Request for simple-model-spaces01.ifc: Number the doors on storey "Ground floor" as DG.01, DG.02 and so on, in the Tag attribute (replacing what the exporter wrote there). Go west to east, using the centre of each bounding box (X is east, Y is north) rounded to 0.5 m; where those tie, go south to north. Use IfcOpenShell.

First a look at what the model holds.

```python
import ifcopenshell
import ifcopenshell.util.element
import ifcopenshell.util.placement

model = ifcopenshell.open("simple-model-spaces01.ifc")
print(model.schema)
storey = next(s for s in model.by_type("IfcBuildingStorey") if s.Name == "Ground floor")
doors = [e for e in ifcopenshell.util.element.get_decomposition(storey) if e.is_a("IfcDoor")]
for e in sorted(doors, key=lambda e: e.id()):
    origin = ifcopenshell.util.placement.get_local_placement(e.ObjectPlacement)[:3, 3]
    print(e.id(), e.Tag, e.Name, origin.round(2) + 0.0, sep=" | ")
```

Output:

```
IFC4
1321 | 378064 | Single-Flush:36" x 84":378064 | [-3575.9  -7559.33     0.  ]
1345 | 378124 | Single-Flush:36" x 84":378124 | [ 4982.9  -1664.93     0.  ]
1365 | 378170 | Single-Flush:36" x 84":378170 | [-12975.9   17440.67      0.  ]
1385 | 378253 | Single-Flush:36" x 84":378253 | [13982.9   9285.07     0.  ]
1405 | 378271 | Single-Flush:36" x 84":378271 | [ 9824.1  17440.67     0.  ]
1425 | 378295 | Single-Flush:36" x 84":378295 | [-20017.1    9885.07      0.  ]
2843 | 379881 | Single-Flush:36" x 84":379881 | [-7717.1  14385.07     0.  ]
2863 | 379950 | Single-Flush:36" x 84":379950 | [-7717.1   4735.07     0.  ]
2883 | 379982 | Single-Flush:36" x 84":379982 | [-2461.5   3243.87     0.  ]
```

```python
import ifcopenshell
import ifcopenshell.geom
import ifcopenshell.util.element
import ifcopenshell.util.shape

model = ifcopenshell.open("simple-model-spaces01.ifc")
settings = ifcopenshell.geom.settings()
settings.set("use-world-coords", True)


def centre(element):
    shape = ifcopenshell.geom.create_shape(settings, element)
    return ifcopenshell.util.shape.get_bbox_centroid(shape.geometry)


storey = next(s for s in model.by_type("IfcBuildingStorey") if s.Name == "Ground floor")
doors = [e for e in ifcopenshell.util.element.get_decomposition(storey) if e.is_a("IfcDoor")]

# Insertion points can sit at a corner or the storey origin, so sort by the geometry (in metres).
centres = {e: centre(e) for e in doors}
doors.sort(key=lambda e: (round(centres[e][0] / 0.5), centres[e][1]))

for i, e in enumerate(doors, start=1):
    number = f"DG.{i:02d}"
    e.Tag = number
    print(e.id(), number)

model.write("simple-model-spaces01_v2.ifc")
```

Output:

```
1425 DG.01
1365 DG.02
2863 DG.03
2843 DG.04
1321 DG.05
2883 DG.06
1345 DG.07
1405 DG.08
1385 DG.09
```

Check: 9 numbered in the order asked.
